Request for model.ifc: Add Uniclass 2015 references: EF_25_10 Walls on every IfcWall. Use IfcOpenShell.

First a look at what the model holds.

```python
import ifcopenshell

model = ifcopenshell.open("model.ifc")
print(model.schema)
print("classifications:", [c.Name for c in model.by_type("IfcClassification")])
for ifc_class in ("IfcDoor", "IfcRoof", "IfcStair", "IfcWall", "IfcWindow"):
    print(ifc_class, len(model.by_type(ifc_class)))
```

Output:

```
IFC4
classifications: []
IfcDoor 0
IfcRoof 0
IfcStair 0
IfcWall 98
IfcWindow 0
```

```python
import ifcopenshell
import ifcopenshell.api.classification

model = ifcopenshell.open("model.ifc")

system = ifcopenshell.api.classification.add_classification(model, classification="Uniclass 2015")

codes = {
    "IfcWall": ("EF_25_10", "Walls"),
}
for ifc_class, (code, name) in codes.items():
    products = model.by_type(ifc_class)
    ifcopenshell.api.classification.add_reference(
        model, products=products, classification=system, identification=code, name=name
    )
    print(code, len(products))

model.write("model_updated.ifc")
```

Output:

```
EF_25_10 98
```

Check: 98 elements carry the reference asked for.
